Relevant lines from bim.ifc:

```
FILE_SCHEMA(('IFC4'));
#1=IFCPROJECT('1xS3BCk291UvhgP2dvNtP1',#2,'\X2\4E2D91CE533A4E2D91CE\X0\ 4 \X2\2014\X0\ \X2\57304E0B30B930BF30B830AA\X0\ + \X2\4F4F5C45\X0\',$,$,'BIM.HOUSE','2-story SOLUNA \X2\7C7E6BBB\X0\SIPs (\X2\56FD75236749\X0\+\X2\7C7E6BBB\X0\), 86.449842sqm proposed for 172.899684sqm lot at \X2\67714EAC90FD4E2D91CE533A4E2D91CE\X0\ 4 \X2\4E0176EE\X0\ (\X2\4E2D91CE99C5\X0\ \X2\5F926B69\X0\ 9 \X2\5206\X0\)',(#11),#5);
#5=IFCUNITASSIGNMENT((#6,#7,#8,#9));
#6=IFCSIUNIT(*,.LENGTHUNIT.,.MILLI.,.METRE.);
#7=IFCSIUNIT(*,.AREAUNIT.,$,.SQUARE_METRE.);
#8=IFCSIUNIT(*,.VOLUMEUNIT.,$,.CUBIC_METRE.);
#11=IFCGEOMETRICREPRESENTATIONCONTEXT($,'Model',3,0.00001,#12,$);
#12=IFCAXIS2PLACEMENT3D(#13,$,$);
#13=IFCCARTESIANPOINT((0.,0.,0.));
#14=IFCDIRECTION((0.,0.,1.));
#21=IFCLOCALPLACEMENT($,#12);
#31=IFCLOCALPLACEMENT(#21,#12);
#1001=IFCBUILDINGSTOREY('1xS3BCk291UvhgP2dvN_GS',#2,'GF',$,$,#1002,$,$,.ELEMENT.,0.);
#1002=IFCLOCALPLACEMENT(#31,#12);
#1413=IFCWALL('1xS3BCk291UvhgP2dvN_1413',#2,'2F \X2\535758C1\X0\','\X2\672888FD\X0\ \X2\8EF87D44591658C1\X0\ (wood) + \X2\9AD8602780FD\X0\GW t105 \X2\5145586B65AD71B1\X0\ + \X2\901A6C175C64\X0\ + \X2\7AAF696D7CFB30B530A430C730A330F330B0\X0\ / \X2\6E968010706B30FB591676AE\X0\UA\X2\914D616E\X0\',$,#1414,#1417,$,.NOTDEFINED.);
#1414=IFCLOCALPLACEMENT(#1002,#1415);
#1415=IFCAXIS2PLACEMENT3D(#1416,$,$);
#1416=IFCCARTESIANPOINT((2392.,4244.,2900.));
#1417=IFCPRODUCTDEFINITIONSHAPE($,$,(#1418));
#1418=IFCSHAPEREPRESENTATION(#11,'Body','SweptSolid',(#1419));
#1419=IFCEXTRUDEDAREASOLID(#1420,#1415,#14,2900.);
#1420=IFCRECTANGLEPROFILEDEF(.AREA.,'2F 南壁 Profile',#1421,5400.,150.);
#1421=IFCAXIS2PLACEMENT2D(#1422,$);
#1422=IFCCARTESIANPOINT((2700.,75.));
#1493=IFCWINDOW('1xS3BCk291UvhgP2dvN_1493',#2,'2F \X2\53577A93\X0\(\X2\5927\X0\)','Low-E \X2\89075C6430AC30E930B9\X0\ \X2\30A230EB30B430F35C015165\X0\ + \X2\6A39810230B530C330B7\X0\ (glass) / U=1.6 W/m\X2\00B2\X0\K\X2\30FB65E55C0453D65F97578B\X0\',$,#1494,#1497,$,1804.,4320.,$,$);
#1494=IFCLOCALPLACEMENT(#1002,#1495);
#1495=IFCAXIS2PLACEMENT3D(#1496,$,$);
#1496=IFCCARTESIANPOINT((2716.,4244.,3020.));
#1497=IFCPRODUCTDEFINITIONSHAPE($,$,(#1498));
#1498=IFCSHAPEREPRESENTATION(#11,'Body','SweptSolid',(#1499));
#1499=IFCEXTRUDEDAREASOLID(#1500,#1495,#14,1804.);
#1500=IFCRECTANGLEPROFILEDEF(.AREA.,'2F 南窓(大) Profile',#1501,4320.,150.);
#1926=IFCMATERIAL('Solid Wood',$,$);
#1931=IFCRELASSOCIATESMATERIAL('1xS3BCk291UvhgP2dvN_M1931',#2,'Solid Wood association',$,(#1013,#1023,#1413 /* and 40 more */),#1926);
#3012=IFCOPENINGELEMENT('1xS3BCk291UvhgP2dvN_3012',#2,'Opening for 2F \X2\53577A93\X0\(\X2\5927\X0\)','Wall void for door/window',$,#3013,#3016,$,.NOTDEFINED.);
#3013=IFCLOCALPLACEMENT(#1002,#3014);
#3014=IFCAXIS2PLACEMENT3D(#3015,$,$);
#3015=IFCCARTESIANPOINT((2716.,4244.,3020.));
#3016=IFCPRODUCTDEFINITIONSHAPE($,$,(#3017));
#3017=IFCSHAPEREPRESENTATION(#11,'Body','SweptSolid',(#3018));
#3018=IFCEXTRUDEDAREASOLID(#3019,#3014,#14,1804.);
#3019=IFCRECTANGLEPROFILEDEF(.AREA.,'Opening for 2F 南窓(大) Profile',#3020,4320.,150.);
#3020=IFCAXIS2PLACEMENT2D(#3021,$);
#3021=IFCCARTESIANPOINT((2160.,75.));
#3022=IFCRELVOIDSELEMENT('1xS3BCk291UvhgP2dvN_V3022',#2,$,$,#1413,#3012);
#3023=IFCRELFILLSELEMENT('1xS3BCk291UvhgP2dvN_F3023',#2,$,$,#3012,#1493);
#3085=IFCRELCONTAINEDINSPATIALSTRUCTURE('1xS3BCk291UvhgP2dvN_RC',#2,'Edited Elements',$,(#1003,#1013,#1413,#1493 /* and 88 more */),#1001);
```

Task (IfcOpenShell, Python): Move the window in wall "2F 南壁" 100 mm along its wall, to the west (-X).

```python
import ifcopenshell
import ifcopenshell.api.geometry
import ifcopenshell.util.placement

model = ifcopenshell.open("bim.ifc")

window = model.by_guid("1xS3BCk291UvhgP2dvN_1493")
opening = window.FillsVoids[0].RelatingOpeningElement
wall = opening.VoidsElements[0].RelatingBuildingElement

wall_matrix = ifcopenshell.util.placement.get_local_placement(wall.ObjectPlacement)
shift = wall_matrix[:3, 0] * -100.0
before = ifcopenshell.util.placement.get_local_placement(window.ObjectPlacement)[:3, 3].copy()

# The window is not placed relative to its opening, so move both.
for product in (opening, window):
    matrix = ifcopenshell.util.placement.get_local_placement(product.ObjectPlacement)
    matrix[:3, 3] += shift
    ifcopenshell.api.geometry.edit_object_placement(model, product=product, matrix=matrix, is_si=False)

after = ifcopenshell.util.placement.get_local_placement(window.ObjectPlacement)[:3, 3]
print("window moved by", (after - before).round(3) + 0.0)

model.write("bim_rev.ifc")
```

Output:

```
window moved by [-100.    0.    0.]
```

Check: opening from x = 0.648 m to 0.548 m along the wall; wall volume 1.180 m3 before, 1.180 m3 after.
